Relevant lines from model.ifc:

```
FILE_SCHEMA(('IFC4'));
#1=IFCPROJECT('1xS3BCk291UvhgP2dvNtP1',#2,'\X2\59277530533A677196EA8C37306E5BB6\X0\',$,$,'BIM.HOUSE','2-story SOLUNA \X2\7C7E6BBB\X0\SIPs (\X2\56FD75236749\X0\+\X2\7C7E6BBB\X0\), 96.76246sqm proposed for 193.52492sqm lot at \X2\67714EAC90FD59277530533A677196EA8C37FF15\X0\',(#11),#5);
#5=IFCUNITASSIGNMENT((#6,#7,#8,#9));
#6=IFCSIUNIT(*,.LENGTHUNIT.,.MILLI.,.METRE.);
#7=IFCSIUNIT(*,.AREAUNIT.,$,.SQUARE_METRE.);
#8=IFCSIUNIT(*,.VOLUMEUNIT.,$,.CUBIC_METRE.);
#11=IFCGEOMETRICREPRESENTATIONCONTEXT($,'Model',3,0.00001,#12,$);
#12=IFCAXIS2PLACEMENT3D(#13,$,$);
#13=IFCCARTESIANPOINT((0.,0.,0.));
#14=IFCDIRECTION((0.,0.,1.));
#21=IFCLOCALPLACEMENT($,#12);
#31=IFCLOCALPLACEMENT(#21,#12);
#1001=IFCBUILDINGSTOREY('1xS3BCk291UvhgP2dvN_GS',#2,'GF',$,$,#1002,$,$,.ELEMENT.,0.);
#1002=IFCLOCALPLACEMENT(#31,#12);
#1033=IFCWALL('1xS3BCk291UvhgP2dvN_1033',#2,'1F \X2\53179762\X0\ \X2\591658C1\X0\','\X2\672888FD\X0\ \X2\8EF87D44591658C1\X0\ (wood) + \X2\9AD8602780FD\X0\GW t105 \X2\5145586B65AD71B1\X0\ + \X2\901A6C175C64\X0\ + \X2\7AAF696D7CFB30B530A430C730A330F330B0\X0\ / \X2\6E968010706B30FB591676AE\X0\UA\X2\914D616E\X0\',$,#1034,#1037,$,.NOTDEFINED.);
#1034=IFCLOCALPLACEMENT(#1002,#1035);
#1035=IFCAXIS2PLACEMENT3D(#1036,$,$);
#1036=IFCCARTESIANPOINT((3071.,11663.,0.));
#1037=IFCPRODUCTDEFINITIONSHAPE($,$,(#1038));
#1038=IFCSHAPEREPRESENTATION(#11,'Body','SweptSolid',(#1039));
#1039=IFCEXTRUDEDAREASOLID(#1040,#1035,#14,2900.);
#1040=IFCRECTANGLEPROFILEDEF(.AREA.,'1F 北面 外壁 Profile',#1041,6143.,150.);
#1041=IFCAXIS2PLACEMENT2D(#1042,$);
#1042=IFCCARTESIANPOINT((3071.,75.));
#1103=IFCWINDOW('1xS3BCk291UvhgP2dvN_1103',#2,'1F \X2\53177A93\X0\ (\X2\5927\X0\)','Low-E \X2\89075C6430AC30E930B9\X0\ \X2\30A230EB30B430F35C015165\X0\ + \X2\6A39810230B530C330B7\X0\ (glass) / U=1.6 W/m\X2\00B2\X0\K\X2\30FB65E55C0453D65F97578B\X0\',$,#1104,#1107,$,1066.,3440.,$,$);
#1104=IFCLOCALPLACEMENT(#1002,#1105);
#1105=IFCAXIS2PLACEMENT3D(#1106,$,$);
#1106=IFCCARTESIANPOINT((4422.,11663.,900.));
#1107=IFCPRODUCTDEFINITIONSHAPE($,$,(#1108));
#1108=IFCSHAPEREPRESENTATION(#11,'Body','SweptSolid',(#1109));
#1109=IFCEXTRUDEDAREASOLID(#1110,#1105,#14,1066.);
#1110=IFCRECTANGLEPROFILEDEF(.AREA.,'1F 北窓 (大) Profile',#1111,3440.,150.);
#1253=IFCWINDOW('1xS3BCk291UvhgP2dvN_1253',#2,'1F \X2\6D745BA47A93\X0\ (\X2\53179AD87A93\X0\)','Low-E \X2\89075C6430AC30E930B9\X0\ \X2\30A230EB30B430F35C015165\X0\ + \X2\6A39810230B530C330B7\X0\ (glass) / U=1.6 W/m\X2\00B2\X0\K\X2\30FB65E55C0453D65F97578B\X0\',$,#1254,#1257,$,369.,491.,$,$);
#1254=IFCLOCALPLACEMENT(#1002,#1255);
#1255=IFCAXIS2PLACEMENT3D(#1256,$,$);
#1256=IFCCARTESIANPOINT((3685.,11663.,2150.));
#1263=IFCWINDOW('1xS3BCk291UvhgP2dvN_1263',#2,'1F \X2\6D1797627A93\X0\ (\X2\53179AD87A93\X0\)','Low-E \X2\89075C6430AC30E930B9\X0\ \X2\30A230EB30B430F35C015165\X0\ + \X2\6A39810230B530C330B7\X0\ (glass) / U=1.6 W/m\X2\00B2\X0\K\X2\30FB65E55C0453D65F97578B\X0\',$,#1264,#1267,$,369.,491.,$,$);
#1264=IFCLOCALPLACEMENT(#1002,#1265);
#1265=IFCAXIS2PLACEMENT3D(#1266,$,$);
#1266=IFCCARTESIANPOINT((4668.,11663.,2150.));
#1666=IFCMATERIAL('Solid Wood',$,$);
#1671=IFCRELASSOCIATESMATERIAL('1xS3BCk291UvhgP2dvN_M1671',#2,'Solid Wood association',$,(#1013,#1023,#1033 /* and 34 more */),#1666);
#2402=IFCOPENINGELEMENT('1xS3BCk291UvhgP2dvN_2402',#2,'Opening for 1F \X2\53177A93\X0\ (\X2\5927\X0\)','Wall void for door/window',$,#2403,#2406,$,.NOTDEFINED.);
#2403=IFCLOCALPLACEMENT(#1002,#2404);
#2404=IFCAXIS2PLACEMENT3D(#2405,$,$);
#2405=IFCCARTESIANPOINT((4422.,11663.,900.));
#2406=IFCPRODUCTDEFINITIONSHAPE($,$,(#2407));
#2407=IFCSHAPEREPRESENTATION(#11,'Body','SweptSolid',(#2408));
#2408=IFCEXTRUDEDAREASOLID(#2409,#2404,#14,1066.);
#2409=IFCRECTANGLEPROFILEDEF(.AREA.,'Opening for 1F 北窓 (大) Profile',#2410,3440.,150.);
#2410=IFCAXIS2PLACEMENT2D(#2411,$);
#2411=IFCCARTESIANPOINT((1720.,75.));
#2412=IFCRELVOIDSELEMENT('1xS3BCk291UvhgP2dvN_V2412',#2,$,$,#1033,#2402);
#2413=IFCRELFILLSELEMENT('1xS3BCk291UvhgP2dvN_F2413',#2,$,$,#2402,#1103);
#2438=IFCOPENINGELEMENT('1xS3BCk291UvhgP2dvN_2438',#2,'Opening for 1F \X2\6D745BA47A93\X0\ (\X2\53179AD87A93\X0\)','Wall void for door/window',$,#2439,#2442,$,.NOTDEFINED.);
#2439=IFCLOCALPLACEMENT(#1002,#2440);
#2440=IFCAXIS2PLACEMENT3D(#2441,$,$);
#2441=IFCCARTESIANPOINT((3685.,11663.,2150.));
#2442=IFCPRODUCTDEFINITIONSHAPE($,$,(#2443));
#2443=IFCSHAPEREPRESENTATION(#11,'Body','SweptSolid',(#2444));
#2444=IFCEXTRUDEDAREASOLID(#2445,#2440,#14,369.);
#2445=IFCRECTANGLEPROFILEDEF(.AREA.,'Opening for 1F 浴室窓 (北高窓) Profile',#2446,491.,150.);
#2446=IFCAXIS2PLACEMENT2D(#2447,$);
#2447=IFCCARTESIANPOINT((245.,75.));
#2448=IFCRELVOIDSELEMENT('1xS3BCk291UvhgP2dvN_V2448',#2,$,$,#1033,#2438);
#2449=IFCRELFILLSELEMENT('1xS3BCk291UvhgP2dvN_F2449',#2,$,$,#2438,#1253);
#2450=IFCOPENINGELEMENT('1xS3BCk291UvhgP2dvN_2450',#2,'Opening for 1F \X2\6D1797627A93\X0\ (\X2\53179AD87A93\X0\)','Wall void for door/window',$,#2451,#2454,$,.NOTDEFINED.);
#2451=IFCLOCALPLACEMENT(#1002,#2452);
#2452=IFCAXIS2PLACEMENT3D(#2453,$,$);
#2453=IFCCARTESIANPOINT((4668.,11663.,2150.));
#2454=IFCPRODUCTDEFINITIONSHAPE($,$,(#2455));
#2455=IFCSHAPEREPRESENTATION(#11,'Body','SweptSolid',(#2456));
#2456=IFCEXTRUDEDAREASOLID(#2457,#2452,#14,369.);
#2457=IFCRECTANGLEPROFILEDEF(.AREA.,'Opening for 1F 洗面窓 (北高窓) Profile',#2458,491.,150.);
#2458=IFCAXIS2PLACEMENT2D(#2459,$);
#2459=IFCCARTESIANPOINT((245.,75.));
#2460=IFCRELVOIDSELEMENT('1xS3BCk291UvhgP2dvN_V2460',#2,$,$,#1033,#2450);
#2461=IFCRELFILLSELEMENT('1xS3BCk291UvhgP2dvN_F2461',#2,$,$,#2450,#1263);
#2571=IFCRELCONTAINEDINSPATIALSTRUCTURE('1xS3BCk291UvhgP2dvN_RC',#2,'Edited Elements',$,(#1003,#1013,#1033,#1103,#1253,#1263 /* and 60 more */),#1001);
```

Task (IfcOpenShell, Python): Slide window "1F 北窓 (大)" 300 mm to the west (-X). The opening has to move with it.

```python
import ifcopenshell
import ifcopenshell.api.geometry
import ifcopenshell.util.placement
import ifcopenshell.util.unit

model = ifcopenshell.open("model.ifc")
unit_scale = ifcopenshell.util.unit.calculate_unit_scale(model)

window = model.by_id(1103)
opening = window.FillsVoids[0].RelatingOpeningElement
wall = opening.VoidsElements[0].RelatingBuildingElement

wall_matrix = ifcopenshell.util.placement.get_local_placement(wall.ObjectPlacement)
shift = wall_matrix[:3, 0] * -0.3 / unit_scale
before = ifcopenshell.util.placement.get_local_placement(window.ObjectPlacement)[:3, 3].copy()

# The window is not placed relative to its opening, so move both.
for product in (opening, window):
    matrix = ifcopenshell.util.placement.get_local_placement(product.ObjectPlacement)
    matrix[:3, 3] += shift
    ifcopenshell.api.geometry.edit_object_placement(model, product=product, matrix=matrix, is_si=False)

after = ifcopenshell.util.placement.get_local_placement(window.ObjectPlacement)[:3, 3]
print("window moved by", (after - before).round(3) + 0.0)

model.write("model-out.ifc")
```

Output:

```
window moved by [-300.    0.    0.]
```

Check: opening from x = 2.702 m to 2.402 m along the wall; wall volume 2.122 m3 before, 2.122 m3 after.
